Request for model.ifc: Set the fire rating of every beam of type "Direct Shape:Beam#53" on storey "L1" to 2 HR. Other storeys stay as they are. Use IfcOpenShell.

First a look at what the model holds.

```python
import ifcopenshell
import ifcopenshell.util.element

model = ifcopenshell.open("model.ifc")
print(model.schema)
storey = next(s for s in model.by_type("IfcBuildingStorey") if s.Name == "L1")
beams = [e for e in ifcopenshell.util.element.get_decomposition(storey) if e.is_a("IfcBeam")]
seen = {}
for e in beams:
    element_type = ifcopenshell.util.element.get_type(e)
    key = (element_type.Name if element_type != e and element_type else None, ifcopenshell.util.element.get_pset(e, "Pset_BeamCommon", "FireRating"))
    seen[key] = seen.get(key, 0) + 1
for (name, value), count in sorted(seen.items(), key=str):
    print(count, "x", name, "|", value)
```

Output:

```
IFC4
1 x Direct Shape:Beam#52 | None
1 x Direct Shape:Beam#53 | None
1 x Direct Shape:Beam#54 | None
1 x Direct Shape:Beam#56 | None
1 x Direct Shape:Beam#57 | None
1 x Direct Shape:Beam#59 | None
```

```python
import ifcopenshell
import ifcopenshell.api.pset
import ifcopenshell.util.element

model = ifcopenshell.open("model.ifc")

storey = next(s for s in model.by_type("IfcBuildingStorey") if s.Name == "L1")
beams = [e for e in ifcopenshell.util.element.get_decomposition(storey) if e.is_a("IfcBeam")]

count = 0
for e in beams:
    element_type = ifcopenshell.util.element.get_type(e)
    if element_type in (None, e) or element_type.Name != "Direct Shape:Beam#53":
        continue
    # add_pset returns the element's existing set when there is one.
    pset = ifcopenshell.api.pset.add_pset(model, product=e, name="Pset_BeamCommon")
    ifcopenshell.api.pset.edit_pset(model, pset=pset, properties={"FireRating": "2 HR"})
    count += 1

print(count, "beams updated")

model.write("model_rev.ifc")
```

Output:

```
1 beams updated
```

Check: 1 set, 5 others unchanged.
